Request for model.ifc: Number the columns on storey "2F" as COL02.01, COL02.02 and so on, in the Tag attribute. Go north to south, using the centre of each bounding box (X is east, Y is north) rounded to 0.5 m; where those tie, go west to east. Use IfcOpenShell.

First a look at what the model holds.

```python
import ifcopenshell
import ifcopenshell.util.element
import ifcopenshell.util.placement

model = ifcopenshell.open("model.ifc")
print(model.schema)
storey = next(s for s in model.by_type("IfcBuildingStorey") if s.Name == "2F")
columns = [e for e in ifcopenshell.util.element.get_decomposition(storey) if e.is_a("IfcColumn")]
for e in sorted(columns, key=lambda e: e.id()):
    origin = ifcopenshell.util.placement.get_local_placement(e.ObjectPlacement)[:3, 3]
    print(e.id(), e.Tag, e.Name, origin.round(2) + 0.0, sep=" | ")
```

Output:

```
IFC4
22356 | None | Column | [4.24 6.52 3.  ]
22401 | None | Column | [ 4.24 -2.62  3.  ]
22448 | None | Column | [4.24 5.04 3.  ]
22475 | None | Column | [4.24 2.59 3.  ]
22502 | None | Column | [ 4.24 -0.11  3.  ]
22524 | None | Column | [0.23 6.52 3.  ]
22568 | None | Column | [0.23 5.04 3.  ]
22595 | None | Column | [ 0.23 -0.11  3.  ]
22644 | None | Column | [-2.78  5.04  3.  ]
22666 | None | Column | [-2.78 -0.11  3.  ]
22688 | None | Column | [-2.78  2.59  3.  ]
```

```python
import ifcopenshell
import ifcopenshell.geom
import ifcopenshell.util.element
import ifcopenshell.util.shape

model = ifcopenshell.open("model.ifc")
settings = ifcopenshell.geom.settings()
settings.set("use-world-coords", True)


def centre(element):
    shape = ifcopenshell.geom.create_shape(settings, element)
    return ifcopenshell.util.shape.get_bbox_centroid(shape.geometry)


storey = next(s for s in model.by_type("IfcBuildingStorey") if s.Name == "2F")
columns = [e for e in ifcopenshell.util.element.get_decomposition(storey) if e.is_a("IfcColumn")]

# Insertion points can sit at a corner or the storey origin, so sort by the geometry (in metres).
centres = {e: centre(e) for e in columns}
columns.sort(key=lambda e: (-round(centres[e][1] / 0.5), centres[e][0]))

for i, e in enumerate(columns, start=1):
    number = f"COL02.{i:02d}"
    e.Tag = number
    print(e.id(), number)

model.write("model_updated.ifc")
```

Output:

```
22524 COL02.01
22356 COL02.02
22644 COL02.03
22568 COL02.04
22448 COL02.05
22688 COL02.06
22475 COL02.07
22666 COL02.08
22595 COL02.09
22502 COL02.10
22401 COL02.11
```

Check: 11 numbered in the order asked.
